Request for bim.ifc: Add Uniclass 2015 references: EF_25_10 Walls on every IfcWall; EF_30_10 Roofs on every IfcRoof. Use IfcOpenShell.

First a look at what the model holds.

```python
import ifcopenshell

model = ifcopenshell.open("bim.ifc")
print(model.schema)
print("classifications:", [c.Name for c in model.by_type("IfcClassification")])
for ifc_class in ("IfcDoor", "IfcRoof", "IfcStair", "IfcWall", "IfcWindow"):
    print(ifc_class, len(model.by_type(ifc_class)))
```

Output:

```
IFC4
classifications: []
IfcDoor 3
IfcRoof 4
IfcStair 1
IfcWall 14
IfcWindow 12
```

```python
import ifcopenshell
import ifcopenshell.api.classification

model = ifcopenshell.open("bim.ifc")

system = ifcopenshell.api.classification.add_classification(model, classification="Uniclass 2015")

codes = {
    "IfcWall": ("EF_25_10", "Walls"),
    "IfcRoof": ("EF_30_10", "Roofs"),
}
for ifc_class, (code, name) in codes.items():
    products = model.by_type(ifc_class)
    ifcopenshell.api.classification.add_reference(
        model, products=products, classification=system, identification=code, name=name
    )
    print(code, len(products))

model.write("bim_v2.ifc")
```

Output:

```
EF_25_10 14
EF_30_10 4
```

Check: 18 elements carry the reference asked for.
